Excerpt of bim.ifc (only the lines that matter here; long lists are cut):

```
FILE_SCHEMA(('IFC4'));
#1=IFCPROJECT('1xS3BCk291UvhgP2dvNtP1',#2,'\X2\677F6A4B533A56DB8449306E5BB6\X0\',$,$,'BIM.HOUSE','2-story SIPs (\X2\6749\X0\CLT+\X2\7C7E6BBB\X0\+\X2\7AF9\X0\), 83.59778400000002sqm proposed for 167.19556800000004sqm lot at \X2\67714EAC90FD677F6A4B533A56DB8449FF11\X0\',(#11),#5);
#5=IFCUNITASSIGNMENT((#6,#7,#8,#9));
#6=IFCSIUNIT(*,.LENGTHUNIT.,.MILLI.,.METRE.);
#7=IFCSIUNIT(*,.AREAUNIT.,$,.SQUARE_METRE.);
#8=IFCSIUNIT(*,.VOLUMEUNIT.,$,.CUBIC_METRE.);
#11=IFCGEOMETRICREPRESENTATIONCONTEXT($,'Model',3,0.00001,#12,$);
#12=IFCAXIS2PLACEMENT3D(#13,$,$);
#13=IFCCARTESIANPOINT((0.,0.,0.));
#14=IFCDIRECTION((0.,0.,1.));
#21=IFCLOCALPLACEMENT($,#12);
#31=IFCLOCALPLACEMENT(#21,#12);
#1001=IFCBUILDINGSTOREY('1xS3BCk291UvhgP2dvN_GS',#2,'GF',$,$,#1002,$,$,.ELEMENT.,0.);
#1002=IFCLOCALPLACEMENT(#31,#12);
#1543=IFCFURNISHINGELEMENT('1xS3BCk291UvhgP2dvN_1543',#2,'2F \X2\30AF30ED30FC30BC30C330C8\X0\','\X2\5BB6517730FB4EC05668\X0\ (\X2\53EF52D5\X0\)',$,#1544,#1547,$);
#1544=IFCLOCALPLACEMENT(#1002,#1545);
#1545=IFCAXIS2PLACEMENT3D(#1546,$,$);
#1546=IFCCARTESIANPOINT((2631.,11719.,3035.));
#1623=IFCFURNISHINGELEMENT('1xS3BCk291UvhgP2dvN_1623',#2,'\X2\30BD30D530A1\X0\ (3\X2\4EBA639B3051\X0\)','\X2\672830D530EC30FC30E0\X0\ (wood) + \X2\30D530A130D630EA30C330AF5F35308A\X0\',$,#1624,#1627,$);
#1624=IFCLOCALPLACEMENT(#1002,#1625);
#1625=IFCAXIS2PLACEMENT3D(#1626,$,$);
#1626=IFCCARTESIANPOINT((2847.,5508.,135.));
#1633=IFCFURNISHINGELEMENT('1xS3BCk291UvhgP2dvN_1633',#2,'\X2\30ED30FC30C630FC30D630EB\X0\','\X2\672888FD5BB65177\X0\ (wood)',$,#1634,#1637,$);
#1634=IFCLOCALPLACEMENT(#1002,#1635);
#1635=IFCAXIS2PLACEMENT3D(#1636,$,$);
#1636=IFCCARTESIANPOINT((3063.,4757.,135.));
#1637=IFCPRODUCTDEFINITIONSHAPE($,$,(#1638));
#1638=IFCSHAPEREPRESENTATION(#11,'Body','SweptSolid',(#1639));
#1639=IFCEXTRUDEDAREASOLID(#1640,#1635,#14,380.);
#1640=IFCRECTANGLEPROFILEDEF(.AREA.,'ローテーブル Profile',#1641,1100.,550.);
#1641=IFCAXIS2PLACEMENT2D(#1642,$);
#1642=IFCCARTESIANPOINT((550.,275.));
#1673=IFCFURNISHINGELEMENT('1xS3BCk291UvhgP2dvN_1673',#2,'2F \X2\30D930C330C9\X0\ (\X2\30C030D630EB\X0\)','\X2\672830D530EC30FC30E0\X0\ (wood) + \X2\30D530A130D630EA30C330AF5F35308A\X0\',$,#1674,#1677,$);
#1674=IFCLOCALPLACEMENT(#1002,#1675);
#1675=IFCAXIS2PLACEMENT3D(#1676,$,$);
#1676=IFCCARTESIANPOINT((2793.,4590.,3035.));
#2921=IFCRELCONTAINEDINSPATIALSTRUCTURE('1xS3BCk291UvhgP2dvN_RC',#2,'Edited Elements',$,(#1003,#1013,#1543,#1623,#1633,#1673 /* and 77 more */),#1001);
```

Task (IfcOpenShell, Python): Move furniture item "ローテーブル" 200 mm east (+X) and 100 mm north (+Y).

```python
import ifcopenshell
import ifcopenshell.api.geometry
import ifcopenshell.util.placement

model = ifcopenshell.open("bim.ifc")

item = model.by_guid("1xS3BCk291UvhgP2dvN_1633")
matrix = ifcopenshell.util.placement.get_local_placement(item.ObjectPlacement)
matrix[0, 3] += 200.0
matrix[1, 3] += 100.0
ifcopenshell.api.geometry.edit_object_placement(model, product=item, matrix=matrix, is_si=False)

print(ifcopenshell.util.placement.get_local_placement(item.ObjectPlacement).round(3) + 0.0)

model.write("bim_updated.ifc")
```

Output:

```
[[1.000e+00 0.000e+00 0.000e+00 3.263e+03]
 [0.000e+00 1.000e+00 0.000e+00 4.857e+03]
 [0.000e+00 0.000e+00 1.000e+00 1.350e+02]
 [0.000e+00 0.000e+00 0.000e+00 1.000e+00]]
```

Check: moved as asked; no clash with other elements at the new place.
